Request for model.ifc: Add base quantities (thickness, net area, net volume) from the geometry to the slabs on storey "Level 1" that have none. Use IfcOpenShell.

First a look at what the model holds.

```python
import ifcopenshell
import ifcopenshell.util.element
import ifcopenshell.util.unit

model = ifcopenshell.open("model.ifc")
print(model.schema)
for unit_type in ("LENGTHUNIT", "AREAUNIT", "VOLUMEUNIT"):
    print(unit_type, ifcopenshell.util.unit.calculate_unit_scale(model, unit_type))
storey = next(s for s in model.by_type("IfcBuildingStorey") if s.Name == "Level 1")
slabs = [e for e in ifcopenshell.util.element.get_decomposition(storey) if e.is_a("IfcSlab")]
for e in sorted(slabs, key=lambda e: e.id()):
    print(e.id(), e.is_a(), e.Name, list(ifcopenshell.util.element.get_psets(e, qtos_only=True)), sep=" | ")
```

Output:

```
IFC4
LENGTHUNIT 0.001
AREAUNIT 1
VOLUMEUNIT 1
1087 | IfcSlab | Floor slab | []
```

```python
import ifcopenshell
import ifcopenshell.api.pset
import ifcopenshell.geom
import ifcopenshell.util.element
import ifcopenshell.util.shape
import ifcopenshell.util.unit

model = ifcopenshell.open("model.ifc")
unit_scale = ifcopenshell.util.unit.calculate_unit_scale(model)
area_scale = ifcopenshell.util.unit.calculate_unit_scale(model, "AREAUNIT")
volume_scale = ifcopenshell.util.unit.calculate_unit_scale(model, "VOLUMEUNIT")
settings = ifcopenshell.geom.settings()

storey = next(s for s in model.by_type("IfcBuildingStorey") if s.Name == "Level 1")
slabs = [e for e in ifcopenshell.util.element.get_decomposition(storey) if e.is_a("IfcSlab")]

for e in sorted(slabs, key=lambda e: e.id()):
    if ifcopenshell.util.element.get_psets(e, qtos_only=True, should_inherit=False):
        continue
    # Geometry comes back in metres, in the element's own axes.
    shape = ifcopenshell.geom.create_shape(settings, e)
    values = {
        "Width": ifcopenshell.util.shape.get_z(shape.geometry) / unit_scale,
        "NetArea": ifcopenshell.util.shape.get_footprint_area(shape.geometry) / area_scale,
        "NetVolume": ifcopenshell.util.shape.get_volume(shape.geometry) / volume_scale,
    }
    qto = ifcopenshell.api.pset.add_qto(model, product=e, name="Qto_SlabBaseQuantities")
    ifcopenshell.api.pset.edit_qto(model, qto=qto, properties=values)
    print(e.id(), {k: round(v, 3) for k, v in values.items()})

model.write("model_edited.ifc")
```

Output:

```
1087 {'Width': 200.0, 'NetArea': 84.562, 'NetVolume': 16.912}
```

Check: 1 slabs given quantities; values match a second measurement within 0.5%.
